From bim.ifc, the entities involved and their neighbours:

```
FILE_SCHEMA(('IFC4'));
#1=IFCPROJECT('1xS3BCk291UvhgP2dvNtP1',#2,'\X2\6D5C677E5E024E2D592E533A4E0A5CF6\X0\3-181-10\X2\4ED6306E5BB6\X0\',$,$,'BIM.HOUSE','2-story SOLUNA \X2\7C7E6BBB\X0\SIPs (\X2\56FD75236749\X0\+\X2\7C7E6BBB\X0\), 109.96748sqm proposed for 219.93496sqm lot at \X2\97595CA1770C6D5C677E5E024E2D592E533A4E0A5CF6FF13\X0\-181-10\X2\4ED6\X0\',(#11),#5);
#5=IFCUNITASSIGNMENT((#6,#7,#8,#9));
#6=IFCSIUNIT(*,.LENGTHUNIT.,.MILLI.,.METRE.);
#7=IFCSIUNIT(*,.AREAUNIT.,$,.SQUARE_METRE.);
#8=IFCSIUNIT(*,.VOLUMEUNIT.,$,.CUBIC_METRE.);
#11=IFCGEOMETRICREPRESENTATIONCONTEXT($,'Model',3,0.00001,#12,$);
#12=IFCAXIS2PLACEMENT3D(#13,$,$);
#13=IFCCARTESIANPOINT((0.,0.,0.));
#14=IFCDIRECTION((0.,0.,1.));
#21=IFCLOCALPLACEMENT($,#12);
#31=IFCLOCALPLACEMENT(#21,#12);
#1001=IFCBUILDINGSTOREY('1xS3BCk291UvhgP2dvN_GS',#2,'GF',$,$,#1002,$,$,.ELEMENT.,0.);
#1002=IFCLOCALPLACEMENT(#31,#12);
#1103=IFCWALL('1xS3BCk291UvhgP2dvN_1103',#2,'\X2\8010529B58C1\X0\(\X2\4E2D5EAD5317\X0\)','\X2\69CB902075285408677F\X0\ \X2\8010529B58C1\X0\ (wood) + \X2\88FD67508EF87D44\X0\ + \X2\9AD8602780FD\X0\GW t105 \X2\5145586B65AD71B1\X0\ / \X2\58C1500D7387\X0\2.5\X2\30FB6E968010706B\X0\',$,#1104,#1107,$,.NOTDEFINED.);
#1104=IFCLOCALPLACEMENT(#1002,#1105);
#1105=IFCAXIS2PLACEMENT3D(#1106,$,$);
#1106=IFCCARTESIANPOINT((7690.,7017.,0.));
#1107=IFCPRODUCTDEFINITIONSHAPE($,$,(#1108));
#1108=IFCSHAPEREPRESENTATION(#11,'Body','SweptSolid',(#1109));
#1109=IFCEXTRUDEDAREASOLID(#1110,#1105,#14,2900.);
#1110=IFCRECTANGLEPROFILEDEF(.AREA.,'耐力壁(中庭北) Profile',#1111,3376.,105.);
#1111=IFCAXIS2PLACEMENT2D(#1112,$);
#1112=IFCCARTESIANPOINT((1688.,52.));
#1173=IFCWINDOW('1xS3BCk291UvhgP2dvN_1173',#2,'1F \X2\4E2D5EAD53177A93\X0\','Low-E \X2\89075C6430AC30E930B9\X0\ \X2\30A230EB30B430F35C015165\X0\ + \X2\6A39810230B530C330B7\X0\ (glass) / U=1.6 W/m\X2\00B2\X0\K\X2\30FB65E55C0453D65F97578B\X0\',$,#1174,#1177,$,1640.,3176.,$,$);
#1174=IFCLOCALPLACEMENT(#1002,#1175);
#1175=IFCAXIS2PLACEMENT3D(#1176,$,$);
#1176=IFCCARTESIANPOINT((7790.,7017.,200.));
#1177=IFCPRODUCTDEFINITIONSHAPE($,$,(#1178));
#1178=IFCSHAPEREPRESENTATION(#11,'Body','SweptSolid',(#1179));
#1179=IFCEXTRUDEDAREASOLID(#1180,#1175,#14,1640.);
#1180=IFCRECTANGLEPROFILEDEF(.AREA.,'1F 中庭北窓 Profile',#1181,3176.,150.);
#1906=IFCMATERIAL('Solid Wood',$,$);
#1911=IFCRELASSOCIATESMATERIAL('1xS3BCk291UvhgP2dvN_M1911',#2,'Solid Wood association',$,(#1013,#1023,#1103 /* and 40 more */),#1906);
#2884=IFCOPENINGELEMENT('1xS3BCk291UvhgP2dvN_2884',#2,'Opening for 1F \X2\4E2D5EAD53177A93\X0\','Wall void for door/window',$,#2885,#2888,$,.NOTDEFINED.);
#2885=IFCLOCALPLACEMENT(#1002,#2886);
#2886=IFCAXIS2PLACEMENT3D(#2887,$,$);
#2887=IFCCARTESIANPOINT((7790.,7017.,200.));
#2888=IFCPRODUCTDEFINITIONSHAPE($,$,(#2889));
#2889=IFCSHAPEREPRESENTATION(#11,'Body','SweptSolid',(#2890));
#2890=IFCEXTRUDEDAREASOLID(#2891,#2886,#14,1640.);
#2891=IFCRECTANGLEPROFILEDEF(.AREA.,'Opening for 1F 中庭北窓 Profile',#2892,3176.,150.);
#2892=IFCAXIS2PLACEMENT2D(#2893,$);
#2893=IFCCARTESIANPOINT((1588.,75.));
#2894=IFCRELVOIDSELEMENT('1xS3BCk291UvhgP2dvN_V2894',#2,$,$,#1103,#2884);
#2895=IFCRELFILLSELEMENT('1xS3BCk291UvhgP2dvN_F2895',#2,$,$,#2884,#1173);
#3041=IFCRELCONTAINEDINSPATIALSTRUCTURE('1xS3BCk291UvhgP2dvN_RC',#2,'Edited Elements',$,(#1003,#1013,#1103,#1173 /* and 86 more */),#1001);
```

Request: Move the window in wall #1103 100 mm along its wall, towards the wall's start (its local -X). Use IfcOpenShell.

```python
import ifcopenshell
import ifcopenshell.api.geometry
import ifcopenshell.util.placement
import ifcopenshell.util.unit

model = ifcopenshell.open("bim.ifc")
unit_scale = ifcopenshell.util.unit.calculate_unit_scale(model)

window = model.by_guid("1xS3BCk291UvhgP2dvN_1173")
opening = window.FillsVoids[0].RelatingOpeningElement
wall = opening.VoidsElements[0].RelatingBuildingElement

wall_matrix = ifcopenshell.util.placement.get_local_placement(wall.ObjectPlacement)
shift = wall_matrix[:3, 0] * -0.1 / unit_scale
before = ifcopenshell.util.placement.get_local_placement(window.ObjectPlacement)[:3, 3].copy()

# The window is not placed relative to its opening, so move both.
for product in (opening, window):
    matrix = ifcopenshell.util.placement.get_local_placement(product.ObjectPlacement)
    matrix[:3, 3] += shift
    ifcopenshell.api.geometry.edit_object_placement(model, product=product, matrix=matrix, is_si=False)

after = ifcopenshell.util.placement.get_local_placement(window.ObjectPlacement)[:3, 3]
print("window moved by", (after - before).round(3) + 0.0)

model.write("bim-out.ifc")
```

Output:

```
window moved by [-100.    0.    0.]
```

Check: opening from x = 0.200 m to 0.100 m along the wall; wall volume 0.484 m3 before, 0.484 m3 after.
